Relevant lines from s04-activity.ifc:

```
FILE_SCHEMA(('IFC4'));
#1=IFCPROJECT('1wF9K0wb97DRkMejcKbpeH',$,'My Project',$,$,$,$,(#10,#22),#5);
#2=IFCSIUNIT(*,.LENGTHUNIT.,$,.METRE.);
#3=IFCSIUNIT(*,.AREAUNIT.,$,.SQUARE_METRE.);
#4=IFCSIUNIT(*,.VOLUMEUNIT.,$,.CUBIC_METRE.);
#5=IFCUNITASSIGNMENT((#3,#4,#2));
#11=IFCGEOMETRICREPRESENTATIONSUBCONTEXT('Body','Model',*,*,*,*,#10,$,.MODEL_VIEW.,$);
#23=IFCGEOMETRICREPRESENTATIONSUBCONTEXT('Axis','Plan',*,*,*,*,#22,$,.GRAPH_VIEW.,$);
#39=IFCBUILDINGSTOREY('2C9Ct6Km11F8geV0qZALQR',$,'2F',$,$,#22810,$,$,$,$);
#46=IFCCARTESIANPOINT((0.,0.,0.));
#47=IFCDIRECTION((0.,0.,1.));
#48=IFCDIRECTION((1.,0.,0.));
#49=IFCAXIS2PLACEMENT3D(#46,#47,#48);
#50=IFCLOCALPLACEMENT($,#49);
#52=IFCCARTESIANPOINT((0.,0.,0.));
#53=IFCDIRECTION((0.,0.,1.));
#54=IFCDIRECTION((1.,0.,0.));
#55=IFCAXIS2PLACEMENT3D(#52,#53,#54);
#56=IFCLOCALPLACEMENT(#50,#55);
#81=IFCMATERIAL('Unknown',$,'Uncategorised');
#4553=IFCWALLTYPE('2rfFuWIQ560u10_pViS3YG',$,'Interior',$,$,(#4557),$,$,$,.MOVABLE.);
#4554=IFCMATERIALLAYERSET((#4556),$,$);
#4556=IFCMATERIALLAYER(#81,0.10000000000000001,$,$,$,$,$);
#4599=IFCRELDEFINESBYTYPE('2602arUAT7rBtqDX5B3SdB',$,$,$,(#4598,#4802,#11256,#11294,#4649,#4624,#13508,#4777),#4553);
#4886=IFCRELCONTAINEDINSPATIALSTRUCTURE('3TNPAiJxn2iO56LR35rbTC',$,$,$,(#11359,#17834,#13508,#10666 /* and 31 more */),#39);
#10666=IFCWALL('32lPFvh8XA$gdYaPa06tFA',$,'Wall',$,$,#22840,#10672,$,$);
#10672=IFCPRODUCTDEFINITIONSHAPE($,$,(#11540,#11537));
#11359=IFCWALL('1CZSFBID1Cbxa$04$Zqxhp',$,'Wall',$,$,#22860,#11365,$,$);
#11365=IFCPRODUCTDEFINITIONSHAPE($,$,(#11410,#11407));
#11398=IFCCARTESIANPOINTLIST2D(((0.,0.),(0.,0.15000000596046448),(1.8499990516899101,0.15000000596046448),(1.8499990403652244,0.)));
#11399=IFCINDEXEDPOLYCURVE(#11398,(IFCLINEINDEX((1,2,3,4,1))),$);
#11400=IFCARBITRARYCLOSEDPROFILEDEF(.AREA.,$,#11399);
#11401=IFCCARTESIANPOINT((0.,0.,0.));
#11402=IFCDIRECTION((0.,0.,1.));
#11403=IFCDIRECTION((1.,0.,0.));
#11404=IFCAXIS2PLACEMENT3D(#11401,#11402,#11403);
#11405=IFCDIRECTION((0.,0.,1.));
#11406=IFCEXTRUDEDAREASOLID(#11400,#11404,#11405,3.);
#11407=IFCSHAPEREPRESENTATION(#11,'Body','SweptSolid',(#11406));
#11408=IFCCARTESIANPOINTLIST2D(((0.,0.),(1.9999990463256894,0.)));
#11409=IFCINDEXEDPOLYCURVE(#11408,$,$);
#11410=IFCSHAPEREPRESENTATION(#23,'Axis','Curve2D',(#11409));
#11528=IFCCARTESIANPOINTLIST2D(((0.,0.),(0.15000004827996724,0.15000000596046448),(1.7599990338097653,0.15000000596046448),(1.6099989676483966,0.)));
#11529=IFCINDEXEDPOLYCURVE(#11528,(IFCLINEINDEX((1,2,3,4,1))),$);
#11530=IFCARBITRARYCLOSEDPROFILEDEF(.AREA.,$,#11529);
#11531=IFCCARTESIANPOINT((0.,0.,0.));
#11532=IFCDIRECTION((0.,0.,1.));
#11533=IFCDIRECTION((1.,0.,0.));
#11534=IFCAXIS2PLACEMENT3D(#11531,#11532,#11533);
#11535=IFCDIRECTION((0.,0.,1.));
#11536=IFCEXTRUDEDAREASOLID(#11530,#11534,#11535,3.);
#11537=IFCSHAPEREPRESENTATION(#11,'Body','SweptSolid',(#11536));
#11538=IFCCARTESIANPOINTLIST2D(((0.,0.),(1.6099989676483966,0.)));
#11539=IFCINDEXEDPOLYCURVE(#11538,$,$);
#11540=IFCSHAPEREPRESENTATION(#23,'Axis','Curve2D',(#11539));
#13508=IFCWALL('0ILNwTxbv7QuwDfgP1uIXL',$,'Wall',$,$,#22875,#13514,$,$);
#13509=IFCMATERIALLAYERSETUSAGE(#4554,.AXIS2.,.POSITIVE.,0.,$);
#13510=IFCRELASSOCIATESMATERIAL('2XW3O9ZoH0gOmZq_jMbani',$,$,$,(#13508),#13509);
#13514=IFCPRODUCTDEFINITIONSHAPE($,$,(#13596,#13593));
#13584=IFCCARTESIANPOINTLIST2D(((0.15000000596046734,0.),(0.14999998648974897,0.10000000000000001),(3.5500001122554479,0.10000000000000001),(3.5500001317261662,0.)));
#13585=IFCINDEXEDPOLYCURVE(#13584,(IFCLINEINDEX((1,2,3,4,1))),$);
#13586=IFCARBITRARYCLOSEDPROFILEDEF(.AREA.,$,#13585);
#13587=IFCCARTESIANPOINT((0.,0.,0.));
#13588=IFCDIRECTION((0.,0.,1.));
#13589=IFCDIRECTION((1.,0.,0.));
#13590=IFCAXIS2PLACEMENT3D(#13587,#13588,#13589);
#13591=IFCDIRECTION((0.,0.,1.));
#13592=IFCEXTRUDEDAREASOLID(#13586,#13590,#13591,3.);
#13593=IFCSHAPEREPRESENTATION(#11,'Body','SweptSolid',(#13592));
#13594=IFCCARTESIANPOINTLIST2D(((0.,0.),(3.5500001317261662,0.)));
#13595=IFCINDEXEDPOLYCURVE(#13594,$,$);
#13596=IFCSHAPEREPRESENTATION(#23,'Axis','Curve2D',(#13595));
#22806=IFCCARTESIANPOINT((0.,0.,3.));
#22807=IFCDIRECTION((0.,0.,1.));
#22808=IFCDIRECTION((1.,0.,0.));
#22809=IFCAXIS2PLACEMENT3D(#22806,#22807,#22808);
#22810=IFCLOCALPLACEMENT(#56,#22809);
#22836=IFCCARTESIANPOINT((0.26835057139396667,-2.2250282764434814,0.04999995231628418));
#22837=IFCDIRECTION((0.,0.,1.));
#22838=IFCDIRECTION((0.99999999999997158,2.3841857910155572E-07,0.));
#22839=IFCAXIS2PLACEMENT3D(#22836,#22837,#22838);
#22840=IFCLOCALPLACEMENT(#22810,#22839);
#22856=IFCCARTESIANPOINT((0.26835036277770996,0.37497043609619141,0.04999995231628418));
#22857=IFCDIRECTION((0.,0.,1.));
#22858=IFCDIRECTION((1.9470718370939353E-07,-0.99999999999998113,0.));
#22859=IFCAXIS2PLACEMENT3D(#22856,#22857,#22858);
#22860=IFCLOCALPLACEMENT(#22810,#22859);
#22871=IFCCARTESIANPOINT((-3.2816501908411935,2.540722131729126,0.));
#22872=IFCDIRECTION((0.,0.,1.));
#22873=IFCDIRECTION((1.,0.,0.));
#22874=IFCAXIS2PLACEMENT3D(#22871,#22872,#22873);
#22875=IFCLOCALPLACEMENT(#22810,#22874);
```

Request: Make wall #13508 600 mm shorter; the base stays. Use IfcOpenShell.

```python
import ifcopenshell
import ifcopenshell.geom
import ifcopenshell.util.representation
import ifcopenshell.util.shape
import ifcopenshell.util.unit

model = ifcopenshell.open("s04-activity.ifc")
unit_scale = ifcopenshell.util.unit.calculate_unit_scale(model)
settings = ifcopenshell.geom.settings()


def volume(element):
    """Net volume in cubic metres, openings subtracted."""
    shape = ifcopenshell.geom.create_shape(settings, element)
    return ifcopenshell.util.shape.get_volume(shape.geometry)


wall = model.by_guid("0ILNwTxbv7QuwDfgP1uIXL")
before = volume(wall)

body = ifcopenshell.util.representation.get_representation(wall, "Model", "Body")
solid = body.Items[0]
old_height = solid.Depth
solid.Depth -= 0.6 / unit_scale
after = volume(wall)

print(f"height {old_height:g} -> {solid.Depth:g}, volume {before:.3f} -> {after:.3f} m3")

model.write("s04-activity-out.ifc")
```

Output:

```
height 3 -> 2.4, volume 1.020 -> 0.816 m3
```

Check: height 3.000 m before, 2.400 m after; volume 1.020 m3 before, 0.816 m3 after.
